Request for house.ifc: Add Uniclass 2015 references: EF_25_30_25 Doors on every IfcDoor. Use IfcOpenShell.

First a look at what the model holds.

```python
import ifcopenshell

model = ifcopenshell.open("house.ifc")
print(model.schema)
print("classifications:", [c.Name for c in model.by_type("IfcClassification")])
for ifc_class in ("IfcDoor", "IfcRoof", "IfcStair", "IfcWall", "IfcWindow"):
    print(ifc_class, len(model.by_type(ifc_class)))
```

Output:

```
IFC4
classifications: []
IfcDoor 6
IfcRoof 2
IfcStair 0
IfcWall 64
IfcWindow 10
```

```python
import ifcopenshell
import ifcopenshell.api.classification

model = ifcopenshell.open("house.ifc")

system = ifcopenshell.api.classification.add_classification(model, classification="Uniclass 2015")

codes = {
    "IfcDoor": ("EF_25_30_25", "Doors"),
}
for ifc_class, (code, name) in codes.items():
    products = model.by_type(ifc_class)
    ifcopenshell.api.classification.add_reference(
        model, products=products, classification=system, identification=code, name=name
    )
    print(code, len(products))

model.write("house_updated.ifc")
```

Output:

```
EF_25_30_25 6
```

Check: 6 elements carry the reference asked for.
